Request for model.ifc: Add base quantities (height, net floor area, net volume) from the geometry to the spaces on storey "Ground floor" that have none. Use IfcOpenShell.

First a look at what the model holds.

```python
import ifcopenshell
import ifcopenshell.util.element
import ifcopenshell.util.unit

model = ifcopenshell.open("model.ifc")
print(model.schema)
for unit_type in ("LENGTHUNIT", "AREAUNIT", "VOLUMEUNIT"):
    print(unit_type, ifcopenshell.util.unit.calculate_unit_scale(model, unit_type))
storey = next(s for s in model.by_type("IfcBuildingStorey") if s.Name == "Ground floor")
spaces = [e for e in ifcopenshell.util.element.get_decomposition(storey) if e.is_a("IfcSpace")]
for e in sorted(spaces, key=lambda e: e.id()):
    print(e.id(), e.is_a(), e.Name, list(ifcopenshell.util.element.get_psets(e, qtos_only=True)), sep=" | ")
```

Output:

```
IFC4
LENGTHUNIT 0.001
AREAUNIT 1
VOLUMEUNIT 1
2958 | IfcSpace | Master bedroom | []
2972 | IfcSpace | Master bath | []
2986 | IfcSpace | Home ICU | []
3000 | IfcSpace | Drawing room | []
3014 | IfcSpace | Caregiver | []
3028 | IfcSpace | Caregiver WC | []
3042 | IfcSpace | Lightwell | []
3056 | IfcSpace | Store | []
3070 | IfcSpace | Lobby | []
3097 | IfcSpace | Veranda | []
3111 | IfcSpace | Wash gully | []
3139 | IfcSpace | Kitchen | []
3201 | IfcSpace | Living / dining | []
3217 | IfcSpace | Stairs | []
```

```python
import ifcopenshell
import ifcopenshell.api.pset
import ifcopenshell.geom
import ifcopenshell.util.element
import ifcopenshell.util.shape
import ifcopenshell.util.unit

model = ifcopenshell.open("model.ifc")
unit_scale = ifcopenshell.util.unit.calculate_unit_scale(model)
area_scale = ifcopenshell.util.unit.calculate_unit_scale(model, "AREAUNIT")
volume_scale = ifcopenshell.util.unit.calculate_unit_scale(model, "VOLUMEUNIT")
settings = ifcopenshell.geom.settings()

storey = next(s for s in model.by_type("IfcBuildingStorey") if s.Name == "Ground floor")
spaces = [e for e in ifcopenshell.util.element.get_decomposition(storey) if e.is_a("IfcSpace")]

for e in sorted(spaces, key=lambda e: e.id()):
    if ifcopenshell.util.element.get_psets(e, qtos_only=True, should_inherit=False):
        continue
    # Geometry comes back in metres, in the element's own axes.
    shape = ifcopenshell.geom.create_shape(settings, e)
    values = {
        "Height": ifcopenshell.util.shape.get_z(shape.geometry) / unit_scale,
        "NetFloorArea": ifcopenshell.util.shape.get_footprint_area(shape.geometry) / area_scale,
        "NetVolume": ifcopenshell.util.shape.get_volume(shape.geometry) / volume_scale,
    }
    qto = ifcopenshell.api.pset.add_qto(model, product=e, name="Qto_SpaceBaseQuantities")
    ifcopenshell.api.pset.edit_qto(model, qto=qto, properties=values)
    print(e.id(), {k: round(v, 3) for k, v in values.items()})

model.write("model_edited.ifc")
```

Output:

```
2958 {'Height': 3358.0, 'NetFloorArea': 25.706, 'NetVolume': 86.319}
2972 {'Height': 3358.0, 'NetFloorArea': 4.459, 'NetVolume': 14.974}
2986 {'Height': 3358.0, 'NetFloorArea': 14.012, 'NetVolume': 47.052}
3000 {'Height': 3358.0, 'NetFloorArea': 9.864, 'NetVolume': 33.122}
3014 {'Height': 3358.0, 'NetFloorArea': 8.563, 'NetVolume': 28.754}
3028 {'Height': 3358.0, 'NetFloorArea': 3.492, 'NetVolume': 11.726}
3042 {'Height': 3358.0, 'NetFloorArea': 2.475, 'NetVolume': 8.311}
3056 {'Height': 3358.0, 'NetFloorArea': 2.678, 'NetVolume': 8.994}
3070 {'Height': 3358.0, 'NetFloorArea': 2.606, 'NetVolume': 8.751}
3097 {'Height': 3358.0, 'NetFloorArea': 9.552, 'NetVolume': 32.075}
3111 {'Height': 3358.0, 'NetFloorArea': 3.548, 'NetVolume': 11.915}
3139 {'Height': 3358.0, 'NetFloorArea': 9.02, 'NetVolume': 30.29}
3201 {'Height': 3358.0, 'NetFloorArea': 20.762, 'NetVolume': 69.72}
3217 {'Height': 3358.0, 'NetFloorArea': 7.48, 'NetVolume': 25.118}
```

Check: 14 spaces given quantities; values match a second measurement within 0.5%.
